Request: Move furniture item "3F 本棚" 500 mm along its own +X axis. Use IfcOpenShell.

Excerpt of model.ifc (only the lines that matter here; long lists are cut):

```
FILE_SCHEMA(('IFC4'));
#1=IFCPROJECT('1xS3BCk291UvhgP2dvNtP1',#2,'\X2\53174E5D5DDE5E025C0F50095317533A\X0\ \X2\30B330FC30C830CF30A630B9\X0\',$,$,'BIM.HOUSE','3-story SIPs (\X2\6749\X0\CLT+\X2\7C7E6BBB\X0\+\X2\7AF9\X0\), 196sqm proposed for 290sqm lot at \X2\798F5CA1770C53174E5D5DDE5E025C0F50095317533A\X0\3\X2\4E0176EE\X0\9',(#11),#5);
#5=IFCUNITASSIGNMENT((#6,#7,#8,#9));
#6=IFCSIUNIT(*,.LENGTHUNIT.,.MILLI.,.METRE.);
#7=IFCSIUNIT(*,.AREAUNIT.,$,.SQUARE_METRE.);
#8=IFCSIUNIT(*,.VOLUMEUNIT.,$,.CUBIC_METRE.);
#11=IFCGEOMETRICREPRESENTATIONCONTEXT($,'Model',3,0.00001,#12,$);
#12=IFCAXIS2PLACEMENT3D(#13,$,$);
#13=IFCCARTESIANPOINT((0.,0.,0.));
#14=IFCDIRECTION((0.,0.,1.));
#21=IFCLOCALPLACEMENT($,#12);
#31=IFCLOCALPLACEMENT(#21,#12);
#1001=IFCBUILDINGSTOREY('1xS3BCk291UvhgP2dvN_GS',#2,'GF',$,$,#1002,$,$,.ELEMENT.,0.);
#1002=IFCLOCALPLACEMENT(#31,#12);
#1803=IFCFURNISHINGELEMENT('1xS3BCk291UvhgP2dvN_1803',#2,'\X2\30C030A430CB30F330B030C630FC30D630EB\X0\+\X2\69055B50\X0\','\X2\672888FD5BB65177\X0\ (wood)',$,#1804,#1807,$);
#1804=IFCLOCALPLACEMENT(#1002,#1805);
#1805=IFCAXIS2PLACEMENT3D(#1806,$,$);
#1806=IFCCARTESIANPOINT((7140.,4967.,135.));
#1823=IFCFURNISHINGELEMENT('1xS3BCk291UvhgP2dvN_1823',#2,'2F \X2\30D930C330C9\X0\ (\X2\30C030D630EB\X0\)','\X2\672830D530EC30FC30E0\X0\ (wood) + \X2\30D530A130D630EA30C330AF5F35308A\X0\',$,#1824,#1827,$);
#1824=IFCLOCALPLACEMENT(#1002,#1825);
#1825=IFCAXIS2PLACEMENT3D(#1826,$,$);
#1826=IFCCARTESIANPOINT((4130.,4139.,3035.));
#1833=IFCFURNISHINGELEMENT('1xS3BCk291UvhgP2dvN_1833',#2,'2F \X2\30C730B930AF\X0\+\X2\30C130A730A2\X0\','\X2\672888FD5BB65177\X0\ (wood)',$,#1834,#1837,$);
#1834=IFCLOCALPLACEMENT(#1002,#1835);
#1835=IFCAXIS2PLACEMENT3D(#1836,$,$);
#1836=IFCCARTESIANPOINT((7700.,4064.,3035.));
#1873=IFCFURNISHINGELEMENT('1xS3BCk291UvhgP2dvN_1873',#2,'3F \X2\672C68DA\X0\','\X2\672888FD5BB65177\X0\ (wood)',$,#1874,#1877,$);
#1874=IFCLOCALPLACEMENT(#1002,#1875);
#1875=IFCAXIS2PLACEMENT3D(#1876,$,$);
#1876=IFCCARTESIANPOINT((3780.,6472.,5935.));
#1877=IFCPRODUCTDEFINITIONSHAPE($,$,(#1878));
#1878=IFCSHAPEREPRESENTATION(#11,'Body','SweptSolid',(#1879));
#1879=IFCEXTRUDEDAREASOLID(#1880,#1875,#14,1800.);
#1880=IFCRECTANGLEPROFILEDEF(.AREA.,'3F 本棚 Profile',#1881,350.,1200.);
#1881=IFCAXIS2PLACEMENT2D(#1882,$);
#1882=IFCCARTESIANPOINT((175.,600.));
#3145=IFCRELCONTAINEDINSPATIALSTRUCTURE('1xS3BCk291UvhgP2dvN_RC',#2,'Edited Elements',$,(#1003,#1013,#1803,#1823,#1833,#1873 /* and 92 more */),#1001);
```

```python
import ifcopenshell
import ifcopenshell.api.geometry
import ifcopenshell.util.placement

model = ifcopenshell.open("model.ifc")

item = model.by_id(1873)
matrix = ifcopenshell.util.placement.get_local_placement(item.ObjectPlacement)
matrix[:3, 3] += matrix[:3, 0] * 500.0
ifcopenshell.api.geometry.edit_object_placement(model, product=item, matrix=matrix, is_si=False)

print(ifcopenshell.util.placement.get_local_placement(item.ObjectPlacement).round(3) + 0.0)

model.write("model_v2.ifc")
```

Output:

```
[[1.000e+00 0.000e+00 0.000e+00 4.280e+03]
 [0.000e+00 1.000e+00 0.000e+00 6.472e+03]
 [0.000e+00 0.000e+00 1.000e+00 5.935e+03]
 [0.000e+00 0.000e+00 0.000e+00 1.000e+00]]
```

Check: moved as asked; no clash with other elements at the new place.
